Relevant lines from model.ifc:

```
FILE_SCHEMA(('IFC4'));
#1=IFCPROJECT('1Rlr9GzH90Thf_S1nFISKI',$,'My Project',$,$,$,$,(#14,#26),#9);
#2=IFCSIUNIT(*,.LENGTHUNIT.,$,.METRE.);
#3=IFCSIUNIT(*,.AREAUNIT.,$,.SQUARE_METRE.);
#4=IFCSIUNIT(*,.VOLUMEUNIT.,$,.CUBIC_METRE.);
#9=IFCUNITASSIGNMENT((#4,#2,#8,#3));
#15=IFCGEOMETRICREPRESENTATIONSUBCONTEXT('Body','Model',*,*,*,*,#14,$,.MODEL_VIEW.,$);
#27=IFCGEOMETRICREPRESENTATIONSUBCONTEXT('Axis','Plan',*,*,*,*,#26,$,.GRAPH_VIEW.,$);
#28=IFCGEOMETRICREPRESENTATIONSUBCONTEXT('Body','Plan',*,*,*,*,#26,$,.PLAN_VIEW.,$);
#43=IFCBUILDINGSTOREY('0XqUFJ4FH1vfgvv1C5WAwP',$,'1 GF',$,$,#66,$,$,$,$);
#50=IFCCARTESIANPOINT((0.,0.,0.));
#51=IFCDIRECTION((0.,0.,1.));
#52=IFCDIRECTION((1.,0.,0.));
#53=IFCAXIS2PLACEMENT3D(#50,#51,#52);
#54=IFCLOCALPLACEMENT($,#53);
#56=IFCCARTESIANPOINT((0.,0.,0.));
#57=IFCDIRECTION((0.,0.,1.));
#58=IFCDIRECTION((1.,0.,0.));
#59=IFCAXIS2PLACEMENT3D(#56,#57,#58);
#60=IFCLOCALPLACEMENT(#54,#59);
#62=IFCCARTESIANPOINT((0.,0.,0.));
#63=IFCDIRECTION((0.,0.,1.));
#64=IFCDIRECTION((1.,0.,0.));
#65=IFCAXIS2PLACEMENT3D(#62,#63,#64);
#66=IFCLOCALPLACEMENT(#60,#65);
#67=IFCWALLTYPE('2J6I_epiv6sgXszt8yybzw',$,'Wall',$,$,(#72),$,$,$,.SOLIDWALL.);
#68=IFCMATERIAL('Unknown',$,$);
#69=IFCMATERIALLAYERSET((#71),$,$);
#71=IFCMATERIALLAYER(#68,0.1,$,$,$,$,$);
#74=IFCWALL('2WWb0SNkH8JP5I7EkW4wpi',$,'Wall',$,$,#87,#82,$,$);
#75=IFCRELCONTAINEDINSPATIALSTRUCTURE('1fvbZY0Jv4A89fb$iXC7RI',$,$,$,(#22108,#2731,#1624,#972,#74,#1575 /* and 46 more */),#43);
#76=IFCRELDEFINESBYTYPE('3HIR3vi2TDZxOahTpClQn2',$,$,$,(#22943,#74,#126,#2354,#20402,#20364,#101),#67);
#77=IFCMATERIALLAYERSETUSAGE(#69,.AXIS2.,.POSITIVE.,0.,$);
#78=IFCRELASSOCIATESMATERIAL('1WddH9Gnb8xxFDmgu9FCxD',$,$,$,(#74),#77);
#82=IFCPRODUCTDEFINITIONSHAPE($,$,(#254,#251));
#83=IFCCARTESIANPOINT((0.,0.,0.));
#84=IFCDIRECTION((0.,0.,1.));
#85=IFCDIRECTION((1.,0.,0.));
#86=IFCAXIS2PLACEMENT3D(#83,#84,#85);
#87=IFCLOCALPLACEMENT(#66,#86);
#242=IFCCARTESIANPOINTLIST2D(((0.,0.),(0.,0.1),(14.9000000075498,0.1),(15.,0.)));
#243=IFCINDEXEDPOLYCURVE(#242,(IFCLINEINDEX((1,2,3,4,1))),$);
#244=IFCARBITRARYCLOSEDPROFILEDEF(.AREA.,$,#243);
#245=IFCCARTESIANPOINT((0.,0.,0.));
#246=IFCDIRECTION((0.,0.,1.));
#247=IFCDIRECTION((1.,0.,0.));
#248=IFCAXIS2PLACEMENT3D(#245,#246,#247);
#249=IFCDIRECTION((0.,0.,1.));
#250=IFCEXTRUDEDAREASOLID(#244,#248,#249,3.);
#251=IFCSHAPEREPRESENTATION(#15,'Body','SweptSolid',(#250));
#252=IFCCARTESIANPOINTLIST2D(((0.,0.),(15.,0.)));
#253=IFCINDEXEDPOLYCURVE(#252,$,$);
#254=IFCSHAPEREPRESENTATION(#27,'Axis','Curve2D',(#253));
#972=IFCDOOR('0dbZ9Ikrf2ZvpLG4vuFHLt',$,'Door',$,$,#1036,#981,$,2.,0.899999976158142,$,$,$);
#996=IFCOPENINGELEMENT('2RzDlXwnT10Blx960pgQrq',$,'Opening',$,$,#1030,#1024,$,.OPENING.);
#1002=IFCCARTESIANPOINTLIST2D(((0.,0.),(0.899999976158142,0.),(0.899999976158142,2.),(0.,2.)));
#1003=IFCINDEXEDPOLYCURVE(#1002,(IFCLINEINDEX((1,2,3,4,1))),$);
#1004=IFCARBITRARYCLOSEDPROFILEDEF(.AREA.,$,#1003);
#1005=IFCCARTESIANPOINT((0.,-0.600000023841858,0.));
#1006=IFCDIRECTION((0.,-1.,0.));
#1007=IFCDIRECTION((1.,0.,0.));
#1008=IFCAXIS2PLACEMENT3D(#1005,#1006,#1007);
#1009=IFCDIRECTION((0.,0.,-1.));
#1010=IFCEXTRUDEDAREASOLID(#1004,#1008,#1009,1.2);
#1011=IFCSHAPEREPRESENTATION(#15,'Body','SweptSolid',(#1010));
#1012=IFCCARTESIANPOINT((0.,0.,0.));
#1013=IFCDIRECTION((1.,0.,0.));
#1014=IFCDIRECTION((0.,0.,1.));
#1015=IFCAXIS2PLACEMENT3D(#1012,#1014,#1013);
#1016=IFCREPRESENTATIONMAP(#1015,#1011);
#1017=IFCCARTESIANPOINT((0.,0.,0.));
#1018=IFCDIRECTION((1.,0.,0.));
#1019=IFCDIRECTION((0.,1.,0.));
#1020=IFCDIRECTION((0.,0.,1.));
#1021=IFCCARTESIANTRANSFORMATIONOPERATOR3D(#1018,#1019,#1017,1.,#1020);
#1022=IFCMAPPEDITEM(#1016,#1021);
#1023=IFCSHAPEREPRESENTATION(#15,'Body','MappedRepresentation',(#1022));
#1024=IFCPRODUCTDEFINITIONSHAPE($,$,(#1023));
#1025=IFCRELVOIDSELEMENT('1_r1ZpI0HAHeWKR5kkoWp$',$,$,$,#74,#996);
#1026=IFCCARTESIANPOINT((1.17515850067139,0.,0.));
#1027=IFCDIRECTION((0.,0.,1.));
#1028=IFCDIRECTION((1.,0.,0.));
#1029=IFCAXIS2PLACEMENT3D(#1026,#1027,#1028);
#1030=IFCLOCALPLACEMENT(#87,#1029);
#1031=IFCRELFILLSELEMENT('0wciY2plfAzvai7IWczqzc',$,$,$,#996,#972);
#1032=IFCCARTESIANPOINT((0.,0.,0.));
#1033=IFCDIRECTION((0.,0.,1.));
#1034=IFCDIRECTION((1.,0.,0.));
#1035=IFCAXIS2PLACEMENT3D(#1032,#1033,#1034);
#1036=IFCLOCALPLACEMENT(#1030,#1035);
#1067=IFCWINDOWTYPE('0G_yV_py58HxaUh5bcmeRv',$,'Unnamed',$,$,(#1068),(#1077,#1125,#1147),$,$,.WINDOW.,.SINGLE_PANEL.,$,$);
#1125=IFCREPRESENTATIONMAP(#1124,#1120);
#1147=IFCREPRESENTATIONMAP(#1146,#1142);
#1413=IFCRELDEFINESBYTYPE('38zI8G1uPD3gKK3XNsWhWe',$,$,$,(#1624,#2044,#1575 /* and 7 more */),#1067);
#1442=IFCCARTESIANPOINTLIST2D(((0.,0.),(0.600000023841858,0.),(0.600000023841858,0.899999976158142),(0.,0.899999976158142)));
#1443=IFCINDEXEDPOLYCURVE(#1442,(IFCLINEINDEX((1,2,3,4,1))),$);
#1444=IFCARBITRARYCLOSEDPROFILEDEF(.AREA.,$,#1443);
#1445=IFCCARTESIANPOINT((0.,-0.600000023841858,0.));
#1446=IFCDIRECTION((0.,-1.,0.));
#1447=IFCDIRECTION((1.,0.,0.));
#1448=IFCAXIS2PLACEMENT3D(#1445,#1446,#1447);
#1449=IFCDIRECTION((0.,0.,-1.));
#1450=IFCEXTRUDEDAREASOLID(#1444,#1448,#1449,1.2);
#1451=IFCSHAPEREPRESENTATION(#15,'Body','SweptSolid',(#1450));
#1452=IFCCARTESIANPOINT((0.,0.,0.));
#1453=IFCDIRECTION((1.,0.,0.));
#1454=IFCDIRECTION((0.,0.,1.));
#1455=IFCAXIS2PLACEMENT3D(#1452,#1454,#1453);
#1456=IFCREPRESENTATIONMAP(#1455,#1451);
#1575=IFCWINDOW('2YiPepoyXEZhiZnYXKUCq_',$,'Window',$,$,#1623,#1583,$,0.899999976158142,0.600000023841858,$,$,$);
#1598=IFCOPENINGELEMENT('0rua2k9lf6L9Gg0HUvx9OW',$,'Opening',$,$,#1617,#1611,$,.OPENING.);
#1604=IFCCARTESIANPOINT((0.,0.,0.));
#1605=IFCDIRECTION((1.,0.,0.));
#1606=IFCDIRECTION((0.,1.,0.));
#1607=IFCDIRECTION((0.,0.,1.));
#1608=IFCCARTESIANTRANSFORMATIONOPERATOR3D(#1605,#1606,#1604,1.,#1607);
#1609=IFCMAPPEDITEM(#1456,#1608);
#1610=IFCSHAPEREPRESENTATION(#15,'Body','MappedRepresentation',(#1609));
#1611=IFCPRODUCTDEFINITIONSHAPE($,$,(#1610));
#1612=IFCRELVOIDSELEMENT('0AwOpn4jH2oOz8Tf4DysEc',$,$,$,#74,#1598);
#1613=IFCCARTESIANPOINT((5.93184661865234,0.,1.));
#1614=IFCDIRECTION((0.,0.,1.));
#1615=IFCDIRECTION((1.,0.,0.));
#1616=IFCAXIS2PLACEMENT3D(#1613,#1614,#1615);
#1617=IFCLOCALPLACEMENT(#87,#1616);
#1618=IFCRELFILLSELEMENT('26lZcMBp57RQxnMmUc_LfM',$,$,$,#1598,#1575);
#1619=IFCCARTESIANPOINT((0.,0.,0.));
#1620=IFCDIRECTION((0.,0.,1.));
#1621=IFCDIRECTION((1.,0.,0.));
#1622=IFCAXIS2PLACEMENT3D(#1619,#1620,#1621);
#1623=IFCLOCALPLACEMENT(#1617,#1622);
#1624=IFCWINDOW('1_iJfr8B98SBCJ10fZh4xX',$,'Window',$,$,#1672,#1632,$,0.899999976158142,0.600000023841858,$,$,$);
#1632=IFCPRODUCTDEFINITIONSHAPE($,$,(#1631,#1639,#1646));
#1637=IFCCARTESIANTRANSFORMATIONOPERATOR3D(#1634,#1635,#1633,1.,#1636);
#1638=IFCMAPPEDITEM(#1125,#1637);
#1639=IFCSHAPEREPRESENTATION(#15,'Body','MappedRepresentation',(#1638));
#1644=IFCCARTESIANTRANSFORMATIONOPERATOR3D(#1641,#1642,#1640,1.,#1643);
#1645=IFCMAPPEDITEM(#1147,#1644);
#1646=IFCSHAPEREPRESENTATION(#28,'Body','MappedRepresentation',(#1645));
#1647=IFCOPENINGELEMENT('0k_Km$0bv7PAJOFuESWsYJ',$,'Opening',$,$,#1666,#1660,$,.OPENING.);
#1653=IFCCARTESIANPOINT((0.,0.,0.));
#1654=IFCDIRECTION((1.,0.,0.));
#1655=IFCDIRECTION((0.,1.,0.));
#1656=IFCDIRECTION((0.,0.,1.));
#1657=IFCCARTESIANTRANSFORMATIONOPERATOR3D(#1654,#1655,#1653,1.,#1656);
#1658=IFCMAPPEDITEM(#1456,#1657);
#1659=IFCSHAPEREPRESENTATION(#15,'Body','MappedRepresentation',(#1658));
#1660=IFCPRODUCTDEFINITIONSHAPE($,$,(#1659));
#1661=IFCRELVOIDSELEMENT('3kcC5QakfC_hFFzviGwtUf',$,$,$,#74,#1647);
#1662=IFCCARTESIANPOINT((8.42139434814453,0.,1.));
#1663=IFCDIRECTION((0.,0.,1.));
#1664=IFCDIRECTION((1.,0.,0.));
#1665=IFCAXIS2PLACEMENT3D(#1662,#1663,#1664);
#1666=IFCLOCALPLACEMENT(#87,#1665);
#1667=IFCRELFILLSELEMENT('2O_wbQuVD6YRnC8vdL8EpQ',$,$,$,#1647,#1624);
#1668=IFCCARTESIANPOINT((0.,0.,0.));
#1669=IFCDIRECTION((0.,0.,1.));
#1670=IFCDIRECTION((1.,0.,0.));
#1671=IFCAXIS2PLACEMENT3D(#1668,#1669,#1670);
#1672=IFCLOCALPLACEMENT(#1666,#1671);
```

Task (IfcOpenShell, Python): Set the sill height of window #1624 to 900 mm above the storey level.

```python
import numpy as np
import ifcopenshell
import ifcopenshell.api.geometry
import ifcopenshell.geom
import ifcopenshell.util.element
import ifcopenshell.util.placement
import ifcopenshell.util.shape
import ifcopenshell.util.unit

model = ifcopenshell.open("model.ifc")
unit_scale = ifcopenshell.util.unit.calculate_unit_scale(model)

window = model.by_guid("1_iJfr8B98SBCJ10fZh4xX")
opening = window.FillsVoids[0].RelatingOpeningElement
storey = ifcopenshell.util.element.get_container(window, ifc_class="IfcBuildingStorey")
level = ifcopenshell.util.placement.get_local_placement(storey.ObjectPlacement)[2, 3]

# The opening's origin need not be at the sill, so measure its lowest point.
shape = ifcopenshell.geom.create_shape(ifcopenshell.geom.settings(), opening)
bottom = ifcopenshell.util.shape.get_shape_bottom_elevation(shape, shape.geometry) / unit_scale
dz = level + 0.9 - bottom

shift = np.array([0.0, 0.0, dz])
# The window is placed relative to its opening, so it follows when the opening moves.
matrix = ifcopenshell.util.placement.get_local_placement(opening.ObjectPlacement)
matrix[:3, 3] += shift
ifcopenshell.api.geometry.edit_object_placement(
    model, product=opening, matrix=matrix, is_si=False, should_transform_children=True
)

print(f"moved by {dz * unit_scale:+.3f} m")

model.write("model_rev.ifc")
```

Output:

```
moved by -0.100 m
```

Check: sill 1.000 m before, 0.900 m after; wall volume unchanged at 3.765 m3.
